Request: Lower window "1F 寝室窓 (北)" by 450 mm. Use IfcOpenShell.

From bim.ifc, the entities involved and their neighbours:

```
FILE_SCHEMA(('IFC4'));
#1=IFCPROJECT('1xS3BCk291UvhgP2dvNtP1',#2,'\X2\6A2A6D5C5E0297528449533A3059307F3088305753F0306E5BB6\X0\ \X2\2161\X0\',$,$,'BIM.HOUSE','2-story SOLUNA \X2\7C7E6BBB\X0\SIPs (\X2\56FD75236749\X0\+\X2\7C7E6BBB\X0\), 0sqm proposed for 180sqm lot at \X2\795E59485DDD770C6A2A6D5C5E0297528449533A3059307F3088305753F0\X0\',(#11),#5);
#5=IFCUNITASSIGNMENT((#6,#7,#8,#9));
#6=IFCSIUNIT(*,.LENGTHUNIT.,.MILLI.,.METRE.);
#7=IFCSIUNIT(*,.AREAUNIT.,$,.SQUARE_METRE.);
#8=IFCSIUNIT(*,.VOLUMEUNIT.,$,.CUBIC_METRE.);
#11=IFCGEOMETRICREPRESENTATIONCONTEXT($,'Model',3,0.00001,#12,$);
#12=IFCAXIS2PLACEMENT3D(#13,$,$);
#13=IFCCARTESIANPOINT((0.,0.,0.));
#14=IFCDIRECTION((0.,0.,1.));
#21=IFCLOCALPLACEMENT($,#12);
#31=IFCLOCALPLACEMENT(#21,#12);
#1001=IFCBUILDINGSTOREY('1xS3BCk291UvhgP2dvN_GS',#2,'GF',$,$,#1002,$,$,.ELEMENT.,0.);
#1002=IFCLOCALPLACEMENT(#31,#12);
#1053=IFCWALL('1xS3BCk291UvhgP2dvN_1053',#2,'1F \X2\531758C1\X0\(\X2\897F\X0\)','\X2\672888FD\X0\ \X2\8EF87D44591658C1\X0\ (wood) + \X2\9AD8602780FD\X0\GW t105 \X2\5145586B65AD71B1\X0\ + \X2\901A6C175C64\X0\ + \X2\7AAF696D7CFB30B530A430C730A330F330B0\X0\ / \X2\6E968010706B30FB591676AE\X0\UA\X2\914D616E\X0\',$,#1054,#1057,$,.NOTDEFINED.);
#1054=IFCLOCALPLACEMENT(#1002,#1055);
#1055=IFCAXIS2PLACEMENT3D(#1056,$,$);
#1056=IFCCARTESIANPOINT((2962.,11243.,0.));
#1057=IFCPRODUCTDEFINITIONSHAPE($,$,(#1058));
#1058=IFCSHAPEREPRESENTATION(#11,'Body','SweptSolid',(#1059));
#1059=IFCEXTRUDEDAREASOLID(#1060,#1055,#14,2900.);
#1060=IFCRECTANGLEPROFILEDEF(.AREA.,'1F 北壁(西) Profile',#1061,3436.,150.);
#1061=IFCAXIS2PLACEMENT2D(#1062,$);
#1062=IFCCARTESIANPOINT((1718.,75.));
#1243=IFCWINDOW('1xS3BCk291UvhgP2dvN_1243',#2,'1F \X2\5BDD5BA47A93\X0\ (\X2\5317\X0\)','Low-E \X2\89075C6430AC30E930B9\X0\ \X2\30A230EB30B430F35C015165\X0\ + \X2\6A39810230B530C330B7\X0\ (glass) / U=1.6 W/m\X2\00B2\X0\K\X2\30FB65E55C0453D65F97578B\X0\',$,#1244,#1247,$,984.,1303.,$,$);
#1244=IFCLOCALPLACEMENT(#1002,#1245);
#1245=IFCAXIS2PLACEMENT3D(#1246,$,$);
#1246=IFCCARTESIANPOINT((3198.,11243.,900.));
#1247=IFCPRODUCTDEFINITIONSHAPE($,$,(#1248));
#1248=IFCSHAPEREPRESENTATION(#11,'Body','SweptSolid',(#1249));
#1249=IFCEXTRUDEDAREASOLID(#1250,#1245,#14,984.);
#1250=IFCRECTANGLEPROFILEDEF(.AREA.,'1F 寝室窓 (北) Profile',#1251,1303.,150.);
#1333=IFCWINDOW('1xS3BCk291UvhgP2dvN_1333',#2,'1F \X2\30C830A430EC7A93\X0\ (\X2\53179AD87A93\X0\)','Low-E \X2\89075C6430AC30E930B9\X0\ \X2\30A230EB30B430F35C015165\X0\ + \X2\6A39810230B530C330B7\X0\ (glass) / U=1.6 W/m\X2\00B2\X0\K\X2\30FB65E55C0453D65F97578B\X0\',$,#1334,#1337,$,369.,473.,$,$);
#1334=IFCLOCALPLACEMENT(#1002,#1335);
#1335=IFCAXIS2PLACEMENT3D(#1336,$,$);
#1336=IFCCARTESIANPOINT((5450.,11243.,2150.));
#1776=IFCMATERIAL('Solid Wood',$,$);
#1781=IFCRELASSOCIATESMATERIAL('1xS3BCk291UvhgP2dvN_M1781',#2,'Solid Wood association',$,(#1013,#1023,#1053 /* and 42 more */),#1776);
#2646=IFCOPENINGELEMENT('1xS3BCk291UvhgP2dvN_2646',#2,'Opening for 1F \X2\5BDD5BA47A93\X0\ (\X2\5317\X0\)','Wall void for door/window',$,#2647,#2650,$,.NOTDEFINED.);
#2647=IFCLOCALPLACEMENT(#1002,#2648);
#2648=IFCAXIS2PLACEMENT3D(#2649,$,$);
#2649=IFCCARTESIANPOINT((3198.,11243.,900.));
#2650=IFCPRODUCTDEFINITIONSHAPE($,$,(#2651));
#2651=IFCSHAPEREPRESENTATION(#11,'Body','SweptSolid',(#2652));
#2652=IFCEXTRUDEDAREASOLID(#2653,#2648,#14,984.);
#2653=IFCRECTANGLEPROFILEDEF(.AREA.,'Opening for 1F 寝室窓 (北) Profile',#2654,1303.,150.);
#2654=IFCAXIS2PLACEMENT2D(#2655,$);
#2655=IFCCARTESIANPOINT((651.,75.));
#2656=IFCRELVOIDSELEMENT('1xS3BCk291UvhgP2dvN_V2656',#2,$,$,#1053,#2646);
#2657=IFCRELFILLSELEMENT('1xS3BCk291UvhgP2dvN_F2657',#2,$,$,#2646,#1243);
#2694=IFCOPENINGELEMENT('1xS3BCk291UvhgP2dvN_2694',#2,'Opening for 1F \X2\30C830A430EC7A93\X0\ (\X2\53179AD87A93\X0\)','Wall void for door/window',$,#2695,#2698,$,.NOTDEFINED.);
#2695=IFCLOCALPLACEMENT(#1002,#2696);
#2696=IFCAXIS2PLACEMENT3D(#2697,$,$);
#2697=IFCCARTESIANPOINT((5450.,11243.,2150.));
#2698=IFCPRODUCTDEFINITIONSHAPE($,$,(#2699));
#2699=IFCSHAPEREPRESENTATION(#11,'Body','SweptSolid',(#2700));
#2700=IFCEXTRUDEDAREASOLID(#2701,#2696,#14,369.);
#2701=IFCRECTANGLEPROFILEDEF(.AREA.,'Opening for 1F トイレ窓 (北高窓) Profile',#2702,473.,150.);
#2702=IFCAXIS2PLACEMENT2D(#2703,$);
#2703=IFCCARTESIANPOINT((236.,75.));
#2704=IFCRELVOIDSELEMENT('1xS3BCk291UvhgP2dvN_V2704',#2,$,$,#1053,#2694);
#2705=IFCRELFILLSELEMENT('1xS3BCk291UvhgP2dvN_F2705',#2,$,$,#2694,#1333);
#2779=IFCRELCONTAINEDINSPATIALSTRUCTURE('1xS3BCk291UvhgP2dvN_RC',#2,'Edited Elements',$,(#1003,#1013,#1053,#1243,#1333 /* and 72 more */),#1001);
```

```python
import numpy as np
import ifcopenshell
import ifcopenshell.api.geometry
import ifcopenshell.util.placement
import ifcopenshell.util.unit

model = ifcopenshell.open("bim.ifc")
unit_scale = ifcopenshell.util.unit.calculate_unit_scale(model)

window = model.by_guid("1xS3BCk291UvhgP2dvN_1243")
opening = window.FillsVoids[0].RelatingOpeningElement
dz = -0.45 / unit_scale

shift = np.array([0.0, 0.0, dz])
# The window is not placed relative to its opening, so move both.
for product in (opening, window):
    matrix = ifcopenshell.util.placement.get_local_placement(product.ObjectPlacement)
    matrix[:3, 3] += shift
    ifcopenshell.api.geometry.edit_object_placement(model, product=product, matrix=matrix, is_si=False)

print(f"moved by {dz * unit_scale:+.3f} m")

model.write("bim-out.ifc")
```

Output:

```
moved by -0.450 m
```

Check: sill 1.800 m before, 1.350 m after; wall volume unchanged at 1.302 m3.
